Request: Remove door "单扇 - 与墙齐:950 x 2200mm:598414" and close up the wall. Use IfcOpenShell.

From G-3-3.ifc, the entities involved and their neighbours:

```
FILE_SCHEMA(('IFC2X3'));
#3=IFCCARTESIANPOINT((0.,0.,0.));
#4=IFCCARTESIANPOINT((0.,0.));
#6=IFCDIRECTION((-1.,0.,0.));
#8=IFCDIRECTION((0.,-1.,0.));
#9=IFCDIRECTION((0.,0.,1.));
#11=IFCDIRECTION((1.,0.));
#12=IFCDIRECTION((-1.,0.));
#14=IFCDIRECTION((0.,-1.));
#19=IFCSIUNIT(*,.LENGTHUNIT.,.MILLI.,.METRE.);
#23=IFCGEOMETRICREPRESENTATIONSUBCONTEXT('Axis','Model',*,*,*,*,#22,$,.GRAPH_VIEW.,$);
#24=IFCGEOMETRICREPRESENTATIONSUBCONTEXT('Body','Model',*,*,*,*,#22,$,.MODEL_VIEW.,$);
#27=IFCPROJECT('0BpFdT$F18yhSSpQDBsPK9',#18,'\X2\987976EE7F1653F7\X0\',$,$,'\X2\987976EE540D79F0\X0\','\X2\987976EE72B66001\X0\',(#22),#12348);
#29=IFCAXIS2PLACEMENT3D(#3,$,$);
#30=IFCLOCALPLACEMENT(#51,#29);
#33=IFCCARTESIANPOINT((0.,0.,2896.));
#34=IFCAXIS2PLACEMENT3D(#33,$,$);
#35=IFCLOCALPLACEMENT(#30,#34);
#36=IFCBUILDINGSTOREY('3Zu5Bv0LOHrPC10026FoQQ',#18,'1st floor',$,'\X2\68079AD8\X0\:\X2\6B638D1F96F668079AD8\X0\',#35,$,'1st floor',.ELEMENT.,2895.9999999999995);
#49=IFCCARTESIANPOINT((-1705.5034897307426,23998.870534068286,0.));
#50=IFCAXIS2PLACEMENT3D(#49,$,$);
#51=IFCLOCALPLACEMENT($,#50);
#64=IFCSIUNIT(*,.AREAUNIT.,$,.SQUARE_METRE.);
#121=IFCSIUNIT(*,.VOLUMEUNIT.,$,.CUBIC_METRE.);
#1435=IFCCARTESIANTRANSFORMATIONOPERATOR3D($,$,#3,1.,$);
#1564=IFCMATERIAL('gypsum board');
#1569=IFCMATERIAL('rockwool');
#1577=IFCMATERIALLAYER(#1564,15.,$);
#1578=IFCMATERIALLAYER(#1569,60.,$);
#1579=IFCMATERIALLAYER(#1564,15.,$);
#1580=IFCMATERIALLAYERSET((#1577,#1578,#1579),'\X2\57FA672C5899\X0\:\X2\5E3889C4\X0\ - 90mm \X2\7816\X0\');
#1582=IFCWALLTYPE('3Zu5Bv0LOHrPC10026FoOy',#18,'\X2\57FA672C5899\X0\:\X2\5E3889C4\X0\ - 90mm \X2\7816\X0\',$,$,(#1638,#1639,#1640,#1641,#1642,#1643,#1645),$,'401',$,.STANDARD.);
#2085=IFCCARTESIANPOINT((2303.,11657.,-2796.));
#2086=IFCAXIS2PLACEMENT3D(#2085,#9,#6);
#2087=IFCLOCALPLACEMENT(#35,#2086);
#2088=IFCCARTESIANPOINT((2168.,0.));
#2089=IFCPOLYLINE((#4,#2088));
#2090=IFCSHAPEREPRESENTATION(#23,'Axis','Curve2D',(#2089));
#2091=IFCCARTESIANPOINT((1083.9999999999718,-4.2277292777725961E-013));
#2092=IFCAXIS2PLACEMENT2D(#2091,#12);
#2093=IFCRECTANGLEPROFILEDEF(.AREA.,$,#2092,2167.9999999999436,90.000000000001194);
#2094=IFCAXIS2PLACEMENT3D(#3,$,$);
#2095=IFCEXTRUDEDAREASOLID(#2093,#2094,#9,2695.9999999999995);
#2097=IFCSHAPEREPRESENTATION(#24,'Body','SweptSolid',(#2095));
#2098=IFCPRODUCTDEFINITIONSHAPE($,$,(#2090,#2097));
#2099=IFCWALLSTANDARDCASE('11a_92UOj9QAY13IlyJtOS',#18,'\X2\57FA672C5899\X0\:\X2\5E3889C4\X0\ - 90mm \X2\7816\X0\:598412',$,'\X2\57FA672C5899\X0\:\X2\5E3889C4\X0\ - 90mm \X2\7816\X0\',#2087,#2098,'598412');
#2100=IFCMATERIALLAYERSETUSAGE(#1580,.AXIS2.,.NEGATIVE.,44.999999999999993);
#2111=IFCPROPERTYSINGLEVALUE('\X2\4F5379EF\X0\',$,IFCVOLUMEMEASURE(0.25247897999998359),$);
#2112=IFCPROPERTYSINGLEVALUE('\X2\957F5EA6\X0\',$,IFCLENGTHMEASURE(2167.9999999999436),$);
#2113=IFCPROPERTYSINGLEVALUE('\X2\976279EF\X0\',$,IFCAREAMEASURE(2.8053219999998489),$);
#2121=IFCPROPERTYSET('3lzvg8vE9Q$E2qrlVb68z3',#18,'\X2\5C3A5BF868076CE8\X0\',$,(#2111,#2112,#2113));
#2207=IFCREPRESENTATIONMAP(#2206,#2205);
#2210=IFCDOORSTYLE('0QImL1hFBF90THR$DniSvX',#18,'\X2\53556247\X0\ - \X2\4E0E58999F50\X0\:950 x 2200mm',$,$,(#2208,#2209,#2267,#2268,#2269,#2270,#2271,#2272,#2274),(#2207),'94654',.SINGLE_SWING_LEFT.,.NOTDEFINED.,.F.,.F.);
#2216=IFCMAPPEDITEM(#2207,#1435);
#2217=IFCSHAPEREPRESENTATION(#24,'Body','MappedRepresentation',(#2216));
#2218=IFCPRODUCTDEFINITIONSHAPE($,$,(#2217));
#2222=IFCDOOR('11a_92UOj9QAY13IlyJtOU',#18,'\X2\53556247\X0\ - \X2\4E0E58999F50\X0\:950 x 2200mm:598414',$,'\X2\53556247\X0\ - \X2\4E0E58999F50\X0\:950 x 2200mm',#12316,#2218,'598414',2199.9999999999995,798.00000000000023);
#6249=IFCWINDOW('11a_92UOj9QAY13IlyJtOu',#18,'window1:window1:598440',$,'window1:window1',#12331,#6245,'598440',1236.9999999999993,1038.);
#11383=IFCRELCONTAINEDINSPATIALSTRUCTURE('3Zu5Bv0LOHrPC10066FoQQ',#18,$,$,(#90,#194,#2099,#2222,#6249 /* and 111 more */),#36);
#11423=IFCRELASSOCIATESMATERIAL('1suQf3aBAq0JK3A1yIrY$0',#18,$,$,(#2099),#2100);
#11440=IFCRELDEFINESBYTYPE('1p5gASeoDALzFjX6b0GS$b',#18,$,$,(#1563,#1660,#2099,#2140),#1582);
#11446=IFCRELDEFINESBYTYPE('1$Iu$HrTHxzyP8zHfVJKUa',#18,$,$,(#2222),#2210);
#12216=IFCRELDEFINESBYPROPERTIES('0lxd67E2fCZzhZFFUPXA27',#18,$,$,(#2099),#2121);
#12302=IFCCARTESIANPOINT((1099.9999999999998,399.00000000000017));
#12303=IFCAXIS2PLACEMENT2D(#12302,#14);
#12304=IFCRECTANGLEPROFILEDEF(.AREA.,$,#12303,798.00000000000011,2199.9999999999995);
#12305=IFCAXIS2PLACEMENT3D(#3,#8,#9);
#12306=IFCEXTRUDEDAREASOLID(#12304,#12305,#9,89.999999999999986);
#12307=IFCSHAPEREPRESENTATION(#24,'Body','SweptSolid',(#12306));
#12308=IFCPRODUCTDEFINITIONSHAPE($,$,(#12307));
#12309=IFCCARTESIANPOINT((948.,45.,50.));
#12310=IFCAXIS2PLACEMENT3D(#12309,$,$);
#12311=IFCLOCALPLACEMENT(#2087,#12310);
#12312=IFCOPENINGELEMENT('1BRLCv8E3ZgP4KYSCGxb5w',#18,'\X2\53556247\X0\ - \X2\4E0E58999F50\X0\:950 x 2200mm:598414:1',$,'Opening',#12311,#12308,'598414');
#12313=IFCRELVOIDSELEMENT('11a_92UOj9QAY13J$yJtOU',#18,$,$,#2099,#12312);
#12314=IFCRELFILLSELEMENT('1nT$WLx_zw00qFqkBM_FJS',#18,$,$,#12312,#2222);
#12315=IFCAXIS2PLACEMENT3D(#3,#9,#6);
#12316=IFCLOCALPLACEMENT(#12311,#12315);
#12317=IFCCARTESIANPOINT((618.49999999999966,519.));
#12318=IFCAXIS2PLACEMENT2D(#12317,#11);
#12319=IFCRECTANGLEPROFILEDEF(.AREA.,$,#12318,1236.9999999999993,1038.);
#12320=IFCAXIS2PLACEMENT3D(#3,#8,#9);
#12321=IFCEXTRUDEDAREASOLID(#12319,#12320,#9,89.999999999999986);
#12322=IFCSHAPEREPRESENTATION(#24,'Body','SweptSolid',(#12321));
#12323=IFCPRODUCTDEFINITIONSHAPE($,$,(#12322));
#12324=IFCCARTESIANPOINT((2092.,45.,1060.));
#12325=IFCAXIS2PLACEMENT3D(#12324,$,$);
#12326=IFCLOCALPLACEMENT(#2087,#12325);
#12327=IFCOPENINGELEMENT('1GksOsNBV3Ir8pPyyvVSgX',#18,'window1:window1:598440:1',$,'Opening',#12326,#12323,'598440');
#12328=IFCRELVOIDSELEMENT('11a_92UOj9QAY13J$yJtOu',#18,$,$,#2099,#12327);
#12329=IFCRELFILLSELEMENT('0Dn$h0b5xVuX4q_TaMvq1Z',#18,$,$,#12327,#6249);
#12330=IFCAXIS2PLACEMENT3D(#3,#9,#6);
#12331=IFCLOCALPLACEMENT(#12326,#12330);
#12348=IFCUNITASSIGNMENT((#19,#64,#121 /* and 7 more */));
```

```python
import ifcopenshell
import ifcopenshell.api.feature
import ifcopenshell.api.pset
import ifcopenshell.api.root
import ifcopenshell.geom
import ifcopenshell.util.element
import ifcopenshell.util.shape
import ifcopenshell.util.unit

model = ifcopenshell.open("G-3-3.ifc")
area_scale = ifcopenshell.util.unit.calculate_unit_scale(model, "AREAUNIT")
volume_scale = ifcopenshell.util.unit.calculate_unit_scale(model, "VOLUMEUNIT")
settings = ifcopenshell.geom.settings()


def volume(element):
    """Net volume in cubic metres, openings subtracted."""
    shape = ifcopenshell.geom.create_shape(settings, element)
    return ifcopenshell.util.shape.get_volume(shape.geometry)


door = model.by_guid("11a_92UOj9QAY13IlyJtOU")
opening = door.FillsVoids[0].RelatingOpeningElement
wall = opening.VoidsElements[0].RelatingBuildingElement
before = volume(wall)

ifcopenshell.api.root.remove_product(model, product=door)
ifcopenshell.api.feature.remove_feature(model, feature=opening)

after = volume(wall)
thickness = 0.09  # wall thickness in metres

# Update the wall's stored quantities.
pset = model.by_id(ifcopenshell.util.element.get_pset(wall, "尺寸标注", should_inherit=False)["id"])
ifcopenshell.api.pset.edit_pset(model, pset=pset, properties={
    "体积": model.create_entity("IfcVolumeMeasure", after / volume_scale),
    "面积": model.create_entity("IfcAreaMeasure", after / thickness / area_scale),
})

print(f"wall volume {before:.3f} -> {after:.3f} m3")

model.write("G-3-3_edited.ifc")
```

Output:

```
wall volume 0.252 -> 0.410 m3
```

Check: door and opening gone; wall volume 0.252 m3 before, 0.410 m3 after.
